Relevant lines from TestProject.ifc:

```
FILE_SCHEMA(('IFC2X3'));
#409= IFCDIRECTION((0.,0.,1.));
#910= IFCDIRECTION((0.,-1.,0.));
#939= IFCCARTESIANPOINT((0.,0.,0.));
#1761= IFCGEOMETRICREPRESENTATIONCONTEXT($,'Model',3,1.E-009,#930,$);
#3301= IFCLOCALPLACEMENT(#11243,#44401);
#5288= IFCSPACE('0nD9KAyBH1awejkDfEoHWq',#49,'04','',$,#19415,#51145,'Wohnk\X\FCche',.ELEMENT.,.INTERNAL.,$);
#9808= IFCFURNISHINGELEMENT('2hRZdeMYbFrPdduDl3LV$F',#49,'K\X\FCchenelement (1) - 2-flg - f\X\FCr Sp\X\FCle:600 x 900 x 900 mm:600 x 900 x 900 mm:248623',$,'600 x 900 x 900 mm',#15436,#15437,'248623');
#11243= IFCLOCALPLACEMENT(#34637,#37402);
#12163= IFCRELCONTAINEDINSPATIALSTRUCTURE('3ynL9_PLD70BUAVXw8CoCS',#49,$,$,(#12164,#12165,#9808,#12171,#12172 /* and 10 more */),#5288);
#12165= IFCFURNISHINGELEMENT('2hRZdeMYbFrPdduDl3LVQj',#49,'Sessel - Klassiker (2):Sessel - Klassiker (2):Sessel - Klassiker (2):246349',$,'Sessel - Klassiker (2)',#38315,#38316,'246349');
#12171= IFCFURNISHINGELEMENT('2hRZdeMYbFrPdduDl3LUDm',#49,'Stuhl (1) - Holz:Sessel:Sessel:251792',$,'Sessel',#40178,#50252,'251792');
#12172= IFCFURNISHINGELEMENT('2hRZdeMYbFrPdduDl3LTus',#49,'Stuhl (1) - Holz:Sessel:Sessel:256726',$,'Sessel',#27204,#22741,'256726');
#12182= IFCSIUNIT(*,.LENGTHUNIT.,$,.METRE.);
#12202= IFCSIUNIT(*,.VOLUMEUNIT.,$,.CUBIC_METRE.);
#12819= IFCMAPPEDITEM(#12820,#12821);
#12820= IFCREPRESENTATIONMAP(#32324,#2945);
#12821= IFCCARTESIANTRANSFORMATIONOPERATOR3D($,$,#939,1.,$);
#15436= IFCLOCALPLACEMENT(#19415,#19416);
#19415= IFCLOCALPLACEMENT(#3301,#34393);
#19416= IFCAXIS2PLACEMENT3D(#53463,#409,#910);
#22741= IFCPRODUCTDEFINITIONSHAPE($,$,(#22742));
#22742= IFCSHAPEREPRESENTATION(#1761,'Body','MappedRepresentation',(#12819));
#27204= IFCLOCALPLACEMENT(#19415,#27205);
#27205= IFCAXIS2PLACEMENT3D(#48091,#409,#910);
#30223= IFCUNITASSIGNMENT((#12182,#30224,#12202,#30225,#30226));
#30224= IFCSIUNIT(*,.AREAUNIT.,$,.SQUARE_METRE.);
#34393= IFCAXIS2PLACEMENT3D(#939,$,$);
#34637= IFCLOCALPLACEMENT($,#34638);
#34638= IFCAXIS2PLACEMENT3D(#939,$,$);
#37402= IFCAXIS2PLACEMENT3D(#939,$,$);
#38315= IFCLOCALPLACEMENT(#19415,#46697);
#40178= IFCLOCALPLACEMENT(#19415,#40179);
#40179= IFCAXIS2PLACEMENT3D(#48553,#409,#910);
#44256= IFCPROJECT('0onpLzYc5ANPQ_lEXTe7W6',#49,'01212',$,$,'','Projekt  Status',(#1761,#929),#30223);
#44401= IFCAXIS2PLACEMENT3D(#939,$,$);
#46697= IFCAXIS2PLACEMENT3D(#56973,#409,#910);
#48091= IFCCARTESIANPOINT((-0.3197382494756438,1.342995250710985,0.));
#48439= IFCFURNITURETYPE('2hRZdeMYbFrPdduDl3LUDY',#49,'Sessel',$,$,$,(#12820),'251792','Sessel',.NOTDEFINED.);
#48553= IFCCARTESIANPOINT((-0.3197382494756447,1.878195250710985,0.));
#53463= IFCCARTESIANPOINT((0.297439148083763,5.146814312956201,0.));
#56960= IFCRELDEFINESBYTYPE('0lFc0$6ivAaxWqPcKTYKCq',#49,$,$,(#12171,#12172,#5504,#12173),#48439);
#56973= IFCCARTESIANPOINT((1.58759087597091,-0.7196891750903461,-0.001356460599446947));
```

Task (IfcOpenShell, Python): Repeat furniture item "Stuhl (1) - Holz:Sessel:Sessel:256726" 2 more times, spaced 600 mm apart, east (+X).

```python
import numpy as np
import ifcopenshell
import ifcopenshell.api.geometry
import ifcopenshell.api.root
import ifcopenshell.util.element
import ifcopenshell.util.placement
import ifcopenshell.util.unit

model = ifcopenshell.open("TestProject.ifc")
unit_scale = ifcopenshell.util.unit.calculate_unit_scale(model)


def reuse_history(source, copy):
    """copy_class also copies each property set's owner history, people and application; keep the originals."""
    for rel in copy.IsDefinedBy:
        if rel.is_a("IfcRelDefinesByProperties") and (history := rel.RelatingPropertyDefinition.OwnerHistory):
            rel.RelatingPropertyDefinition.OwnerHistory = source.OwnerHistory
            ifcopenshell.util.element.remove_deep2(model, history)


source = model.by_guid("2hRZdeMYbFrPdduDl3LTus")
base = ifcopenshell.util.placement.get_local_placement(source.ObjectPlacement)
step = np.array([1.0, 0.0, 0.0]) * 0.6 / unit_scale

for i in range(1, 3):
    copy = ifcopenshell.api.root.copy_class(model, product=source)
    copy.Representation = ifcopenshell.util.element.copy_deep(
        model, source.Representation, exclude=["IfcGeometricRepresentationContext", "IfcRepresentationMap"]
    )
    copy.Name = "Stuhl (1) - Holz:Sessel:Sessel"
    copy.Tag = None
    reuse_history(source, copy)
    matrix = base.copy()
    matrix[:3, 3] += i * step
    print("added at", matrix[:3, 3].round(3) + 0.0)
    ifcopenshell.api.geometry.edit_object_placement(model, product=copy, matrix=matrix, is_si=False)

model.write("TestProject_edited.ifc")
```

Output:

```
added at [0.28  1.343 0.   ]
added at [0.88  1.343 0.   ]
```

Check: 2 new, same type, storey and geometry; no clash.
